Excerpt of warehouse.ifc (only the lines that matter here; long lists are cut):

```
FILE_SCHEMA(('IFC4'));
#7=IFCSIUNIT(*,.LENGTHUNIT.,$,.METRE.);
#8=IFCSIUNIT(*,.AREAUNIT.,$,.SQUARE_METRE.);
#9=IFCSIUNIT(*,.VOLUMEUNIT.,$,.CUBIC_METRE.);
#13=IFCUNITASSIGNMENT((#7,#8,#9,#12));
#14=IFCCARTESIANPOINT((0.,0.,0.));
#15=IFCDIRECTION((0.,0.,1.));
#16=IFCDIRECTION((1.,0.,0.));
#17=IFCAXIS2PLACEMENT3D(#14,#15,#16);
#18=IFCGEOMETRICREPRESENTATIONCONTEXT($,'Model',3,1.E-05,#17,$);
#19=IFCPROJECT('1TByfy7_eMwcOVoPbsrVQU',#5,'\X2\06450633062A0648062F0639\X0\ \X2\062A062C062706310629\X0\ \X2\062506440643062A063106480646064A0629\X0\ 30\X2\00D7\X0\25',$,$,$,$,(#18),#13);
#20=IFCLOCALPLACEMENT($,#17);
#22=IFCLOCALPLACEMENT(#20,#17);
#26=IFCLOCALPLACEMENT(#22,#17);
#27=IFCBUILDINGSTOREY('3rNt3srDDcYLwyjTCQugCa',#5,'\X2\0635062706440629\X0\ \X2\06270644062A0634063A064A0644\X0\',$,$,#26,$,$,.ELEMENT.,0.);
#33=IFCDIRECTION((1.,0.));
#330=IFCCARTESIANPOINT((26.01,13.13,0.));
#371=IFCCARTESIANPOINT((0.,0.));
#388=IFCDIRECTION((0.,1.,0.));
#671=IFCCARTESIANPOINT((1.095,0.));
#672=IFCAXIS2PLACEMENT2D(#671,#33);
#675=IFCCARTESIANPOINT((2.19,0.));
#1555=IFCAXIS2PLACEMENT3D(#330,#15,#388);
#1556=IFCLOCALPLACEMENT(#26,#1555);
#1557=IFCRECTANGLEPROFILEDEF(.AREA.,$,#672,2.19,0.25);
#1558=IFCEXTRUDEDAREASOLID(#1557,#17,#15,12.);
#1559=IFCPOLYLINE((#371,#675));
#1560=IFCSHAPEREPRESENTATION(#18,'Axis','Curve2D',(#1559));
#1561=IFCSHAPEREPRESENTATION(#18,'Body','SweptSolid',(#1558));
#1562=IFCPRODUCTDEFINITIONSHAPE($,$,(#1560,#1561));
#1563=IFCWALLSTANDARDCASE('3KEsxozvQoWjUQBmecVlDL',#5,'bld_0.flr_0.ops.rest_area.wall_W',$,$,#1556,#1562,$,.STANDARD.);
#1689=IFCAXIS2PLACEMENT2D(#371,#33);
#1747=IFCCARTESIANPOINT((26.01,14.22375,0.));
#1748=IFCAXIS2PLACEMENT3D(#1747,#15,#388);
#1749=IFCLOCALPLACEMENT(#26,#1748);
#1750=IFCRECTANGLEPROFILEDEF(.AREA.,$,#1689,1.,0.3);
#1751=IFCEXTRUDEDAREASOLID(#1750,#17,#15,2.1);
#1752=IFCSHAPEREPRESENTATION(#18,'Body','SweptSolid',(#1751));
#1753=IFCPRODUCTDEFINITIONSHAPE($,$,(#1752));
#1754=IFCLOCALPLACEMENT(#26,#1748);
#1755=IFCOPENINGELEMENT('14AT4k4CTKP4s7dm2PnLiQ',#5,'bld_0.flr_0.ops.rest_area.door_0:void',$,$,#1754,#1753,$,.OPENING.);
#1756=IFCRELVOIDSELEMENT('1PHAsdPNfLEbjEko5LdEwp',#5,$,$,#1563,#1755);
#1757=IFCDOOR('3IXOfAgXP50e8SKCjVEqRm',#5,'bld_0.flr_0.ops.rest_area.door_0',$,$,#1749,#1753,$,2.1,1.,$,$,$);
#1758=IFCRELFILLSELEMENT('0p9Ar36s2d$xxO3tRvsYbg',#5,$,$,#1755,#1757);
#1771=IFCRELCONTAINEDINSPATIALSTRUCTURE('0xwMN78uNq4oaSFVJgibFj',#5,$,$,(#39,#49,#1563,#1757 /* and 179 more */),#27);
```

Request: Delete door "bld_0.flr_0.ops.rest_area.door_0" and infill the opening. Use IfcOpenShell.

```python
import ifcopenshell
import ifcopenshell.api.feature
import ifcopenshell.api.root
import ifcopenshell.geom
import ifcopenshell.util.shape

model = ifcopenshell.open("warehouse.ifc")
settings = ifcopenshell.geom.settings()


def volume(element):
    """Net volume in cubic metres, openings subtracted."""
    shape = ifcopenshell.geom.create_shape(settings, element)
    return ifcopenshell.util.shape.get_volume(shape.geometry)


door = model.by_guid("3IXOfAgXP50e8SKCjVEqRm")
opening = door.FillsVoids[0].RelatingOpeningElement
wall = opening.VoidsElements[0].RelatingBuildingElement
before = volume(wall)

ifcopenshell.api.root.remove_product(model, product=door)
ifcopenshell.api.feature.remove_feature(model, feature=opening)

after = volume(wall)

print(f"wall volume {before:.3f} -> {after:.3f} m3")

model.write("warehouse_updated.ifc")
```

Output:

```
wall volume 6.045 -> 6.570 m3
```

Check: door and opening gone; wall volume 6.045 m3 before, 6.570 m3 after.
